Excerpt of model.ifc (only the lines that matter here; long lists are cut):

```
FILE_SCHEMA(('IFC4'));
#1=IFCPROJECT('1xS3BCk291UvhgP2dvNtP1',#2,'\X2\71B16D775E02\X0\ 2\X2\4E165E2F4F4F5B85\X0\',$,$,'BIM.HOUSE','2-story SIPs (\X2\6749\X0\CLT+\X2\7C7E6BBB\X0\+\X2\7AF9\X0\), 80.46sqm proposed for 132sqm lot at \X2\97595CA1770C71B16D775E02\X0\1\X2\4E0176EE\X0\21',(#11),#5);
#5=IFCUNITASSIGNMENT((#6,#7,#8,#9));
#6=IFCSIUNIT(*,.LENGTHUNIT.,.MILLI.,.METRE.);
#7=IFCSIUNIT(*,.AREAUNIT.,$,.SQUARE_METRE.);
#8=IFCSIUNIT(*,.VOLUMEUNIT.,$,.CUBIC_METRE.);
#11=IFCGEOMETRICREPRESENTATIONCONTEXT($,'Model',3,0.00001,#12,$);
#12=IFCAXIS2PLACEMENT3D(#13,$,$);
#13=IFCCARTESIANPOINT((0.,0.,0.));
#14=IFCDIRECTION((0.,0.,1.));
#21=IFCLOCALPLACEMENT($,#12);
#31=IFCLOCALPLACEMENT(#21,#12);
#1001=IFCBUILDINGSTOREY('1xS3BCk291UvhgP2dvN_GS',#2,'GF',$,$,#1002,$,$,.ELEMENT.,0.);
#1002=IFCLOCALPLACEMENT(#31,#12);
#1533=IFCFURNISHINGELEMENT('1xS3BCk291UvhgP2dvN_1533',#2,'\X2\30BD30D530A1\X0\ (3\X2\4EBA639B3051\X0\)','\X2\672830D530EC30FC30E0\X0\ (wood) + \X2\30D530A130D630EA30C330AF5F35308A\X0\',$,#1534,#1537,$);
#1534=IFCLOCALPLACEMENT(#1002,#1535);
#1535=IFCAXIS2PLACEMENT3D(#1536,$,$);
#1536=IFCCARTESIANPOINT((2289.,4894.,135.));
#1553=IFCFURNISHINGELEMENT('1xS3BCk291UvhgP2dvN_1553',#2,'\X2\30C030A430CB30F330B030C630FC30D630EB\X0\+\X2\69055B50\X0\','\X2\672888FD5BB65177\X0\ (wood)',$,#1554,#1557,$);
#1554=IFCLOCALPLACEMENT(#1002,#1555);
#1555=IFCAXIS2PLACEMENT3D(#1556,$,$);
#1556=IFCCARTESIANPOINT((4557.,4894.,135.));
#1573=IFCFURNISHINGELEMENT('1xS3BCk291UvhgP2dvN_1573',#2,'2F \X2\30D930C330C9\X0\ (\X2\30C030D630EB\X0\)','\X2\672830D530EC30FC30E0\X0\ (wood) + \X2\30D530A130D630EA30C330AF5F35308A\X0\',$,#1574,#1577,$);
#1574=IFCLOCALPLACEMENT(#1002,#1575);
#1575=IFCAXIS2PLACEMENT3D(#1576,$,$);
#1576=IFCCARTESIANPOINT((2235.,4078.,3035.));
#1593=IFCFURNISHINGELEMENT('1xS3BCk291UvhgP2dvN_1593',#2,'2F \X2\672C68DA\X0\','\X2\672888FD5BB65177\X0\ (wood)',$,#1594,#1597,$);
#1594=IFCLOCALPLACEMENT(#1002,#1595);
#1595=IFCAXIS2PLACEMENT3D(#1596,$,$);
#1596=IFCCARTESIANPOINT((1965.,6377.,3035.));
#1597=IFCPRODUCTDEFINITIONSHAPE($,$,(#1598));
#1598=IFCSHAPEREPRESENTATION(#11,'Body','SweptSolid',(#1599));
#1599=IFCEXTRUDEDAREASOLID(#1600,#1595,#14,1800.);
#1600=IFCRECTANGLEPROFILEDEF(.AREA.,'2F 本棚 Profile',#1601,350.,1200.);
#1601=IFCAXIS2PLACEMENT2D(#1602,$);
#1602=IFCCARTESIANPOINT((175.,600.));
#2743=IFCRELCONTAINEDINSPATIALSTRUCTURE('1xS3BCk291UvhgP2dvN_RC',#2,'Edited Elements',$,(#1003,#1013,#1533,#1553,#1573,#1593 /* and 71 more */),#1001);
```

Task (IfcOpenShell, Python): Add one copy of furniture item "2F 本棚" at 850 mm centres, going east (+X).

```python
import numpy as np
import ifcopenshell
import ifcopenshell.api.geometry
import ifcopenshell.api.root
import ifcopenshell.util.element
import ifcopenshell.util.placement

model = ifcopenshell.open("model.ifc")


def reuse_history(source, copy):
    """copy_class also copies each property set's owner history, people and application; keep the originals."""
    for rel in copy.IsDefinedBy:
        if rel.is_a("IfcRelDefinesByProperties") and (history := rel.RelatingPropertyDefinition.OwnerHistory):
            rel.RelatingPropertyDefinition.OwnerHistory = source.OwnerHistory
            ifcopenshell.util.element.remove_deep2(model, history)


source = model.by_id(1593)
base = ifcopenshell.util.placement.get_local_placement(source.ObjectPlacement)
step = np.array([1.0, 0.0, 0.0]) * 850.0

for i in range(1, 2):
    copy = ifcopenshell.api.root.copy_class(model, product=source)
    copy.Representation = ifcopenshell.util.element.copy_deep(
        model, source.Representation, exclude=["IfcGeometricRepresentationContext", "IfcRepresentationMap"]
    )
    reuse_history(source, copy)
    matrix = base.copy()
    matrix[:3, 3] += i * step
    print("added at", matrix[:3, 3].round(3) + 0.0)
    ifcopenshell.api.geometry.edit_object_placement(model, product=copy, matrix=matrix, is_si=False)

model.write("model_edited.ifc")
```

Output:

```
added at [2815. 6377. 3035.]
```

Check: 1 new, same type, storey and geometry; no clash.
